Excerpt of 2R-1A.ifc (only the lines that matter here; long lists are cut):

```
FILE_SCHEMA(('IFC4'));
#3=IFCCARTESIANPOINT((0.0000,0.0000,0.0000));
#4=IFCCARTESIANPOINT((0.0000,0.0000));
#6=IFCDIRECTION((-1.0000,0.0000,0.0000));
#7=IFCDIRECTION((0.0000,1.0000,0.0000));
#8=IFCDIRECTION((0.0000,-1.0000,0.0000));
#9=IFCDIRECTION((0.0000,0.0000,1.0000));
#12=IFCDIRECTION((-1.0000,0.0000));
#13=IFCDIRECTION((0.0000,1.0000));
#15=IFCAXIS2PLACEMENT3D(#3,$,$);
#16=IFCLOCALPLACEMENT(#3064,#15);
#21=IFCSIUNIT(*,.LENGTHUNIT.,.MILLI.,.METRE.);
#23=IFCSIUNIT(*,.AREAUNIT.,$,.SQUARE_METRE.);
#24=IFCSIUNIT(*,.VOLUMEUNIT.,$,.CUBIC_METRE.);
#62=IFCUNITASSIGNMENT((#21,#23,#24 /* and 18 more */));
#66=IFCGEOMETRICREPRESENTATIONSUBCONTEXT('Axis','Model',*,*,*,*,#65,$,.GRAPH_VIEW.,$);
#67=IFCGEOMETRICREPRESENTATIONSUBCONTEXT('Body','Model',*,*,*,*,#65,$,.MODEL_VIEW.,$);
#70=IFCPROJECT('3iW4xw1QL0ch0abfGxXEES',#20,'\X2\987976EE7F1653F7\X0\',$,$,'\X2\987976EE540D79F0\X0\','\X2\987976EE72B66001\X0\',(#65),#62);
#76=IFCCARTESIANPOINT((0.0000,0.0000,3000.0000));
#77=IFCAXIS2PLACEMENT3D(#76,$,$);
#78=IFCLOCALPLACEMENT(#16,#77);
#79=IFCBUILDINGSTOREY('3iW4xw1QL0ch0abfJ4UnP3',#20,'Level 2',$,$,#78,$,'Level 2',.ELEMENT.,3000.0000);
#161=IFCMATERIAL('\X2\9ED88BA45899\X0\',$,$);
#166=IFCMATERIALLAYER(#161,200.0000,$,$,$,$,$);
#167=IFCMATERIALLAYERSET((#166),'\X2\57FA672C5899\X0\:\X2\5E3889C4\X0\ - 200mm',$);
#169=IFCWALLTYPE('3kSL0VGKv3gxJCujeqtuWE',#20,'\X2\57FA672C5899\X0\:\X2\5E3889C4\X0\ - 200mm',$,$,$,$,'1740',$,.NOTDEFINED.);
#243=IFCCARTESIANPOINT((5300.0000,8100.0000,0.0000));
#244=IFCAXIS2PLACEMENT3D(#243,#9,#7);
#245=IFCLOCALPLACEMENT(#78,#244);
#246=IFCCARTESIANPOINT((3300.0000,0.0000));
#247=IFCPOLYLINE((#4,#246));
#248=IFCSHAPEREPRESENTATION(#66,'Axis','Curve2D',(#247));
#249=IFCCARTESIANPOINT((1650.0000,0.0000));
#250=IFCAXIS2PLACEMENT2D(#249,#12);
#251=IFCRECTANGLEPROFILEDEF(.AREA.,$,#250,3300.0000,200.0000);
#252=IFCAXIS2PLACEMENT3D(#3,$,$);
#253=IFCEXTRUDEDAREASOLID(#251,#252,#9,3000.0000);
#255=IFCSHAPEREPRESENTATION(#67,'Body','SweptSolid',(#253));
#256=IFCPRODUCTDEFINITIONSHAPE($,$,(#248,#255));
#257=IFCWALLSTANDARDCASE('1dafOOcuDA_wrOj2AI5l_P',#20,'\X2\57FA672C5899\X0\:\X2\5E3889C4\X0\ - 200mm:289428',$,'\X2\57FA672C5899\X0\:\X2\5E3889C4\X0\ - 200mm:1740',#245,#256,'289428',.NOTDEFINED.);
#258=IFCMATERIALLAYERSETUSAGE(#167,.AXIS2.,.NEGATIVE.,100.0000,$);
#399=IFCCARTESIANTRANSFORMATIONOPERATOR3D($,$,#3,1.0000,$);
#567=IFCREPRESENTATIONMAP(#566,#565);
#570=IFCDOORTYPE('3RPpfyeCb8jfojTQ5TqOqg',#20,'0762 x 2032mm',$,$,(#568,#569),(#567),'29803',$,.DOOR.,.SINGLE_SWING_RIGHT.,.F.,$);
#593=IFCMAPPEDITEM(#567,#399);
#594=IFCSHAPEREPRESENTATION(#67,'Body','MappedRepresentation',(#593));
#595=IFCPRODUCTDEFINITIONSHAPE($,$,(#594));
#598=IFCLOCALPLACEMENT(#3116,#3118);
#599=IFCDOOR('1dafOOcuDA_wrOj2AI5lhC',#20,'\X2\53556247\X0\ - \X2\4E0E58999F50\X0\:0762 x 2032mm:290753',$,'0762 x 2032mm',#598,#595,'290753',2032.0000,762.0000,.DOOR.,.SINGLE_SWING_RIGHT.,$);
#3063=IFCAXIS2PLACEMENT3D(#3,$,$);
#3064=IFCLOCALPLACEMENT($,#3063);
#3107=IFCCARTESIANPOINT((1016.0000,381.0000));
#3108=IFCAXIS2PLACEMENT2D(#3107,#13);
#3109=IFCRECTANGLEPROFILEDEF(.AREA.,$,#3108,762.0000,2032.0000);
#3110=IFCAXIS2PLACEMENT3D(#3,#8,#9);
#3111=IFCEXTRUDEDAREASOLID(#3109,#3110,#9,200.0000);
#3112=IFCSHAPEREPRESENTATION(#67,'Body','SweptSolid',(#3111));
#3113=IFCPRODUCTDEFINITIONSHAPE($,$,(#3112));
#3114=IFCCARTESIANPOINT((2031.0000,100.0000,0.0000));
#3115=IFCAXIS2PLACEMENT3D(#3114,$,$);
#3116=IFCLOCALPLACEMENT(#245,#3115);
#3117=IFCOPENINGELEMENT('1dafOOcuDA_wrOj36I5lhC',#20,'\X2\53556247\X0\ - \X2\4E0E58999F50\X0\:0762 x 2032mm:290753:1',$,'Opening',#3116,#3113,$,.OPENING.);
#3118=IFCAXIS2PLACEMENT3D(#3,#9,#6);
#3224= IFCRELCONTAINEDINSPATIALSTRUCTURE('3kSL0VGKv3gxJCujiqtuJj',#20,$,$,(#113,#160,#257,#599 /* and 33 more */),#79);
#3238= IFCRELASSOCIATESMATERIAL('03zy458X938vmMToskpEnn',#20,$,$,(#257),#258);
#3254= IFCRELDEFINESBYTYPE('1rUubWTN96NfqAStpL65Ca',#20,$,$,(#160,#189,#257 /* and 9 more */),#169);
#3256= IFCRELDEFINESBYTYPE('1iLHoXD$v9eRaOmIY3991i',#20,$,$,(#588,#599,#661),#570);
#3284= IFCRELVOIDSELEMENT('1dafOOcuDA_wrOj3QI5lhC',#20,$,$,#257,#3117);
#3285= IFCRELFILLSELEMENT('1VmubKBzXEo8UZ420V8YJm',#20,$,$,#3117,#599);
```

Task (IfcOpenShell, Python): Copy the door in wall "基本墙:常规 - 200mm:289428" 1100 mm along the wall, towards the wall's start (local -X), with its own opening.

```python
import ifcopenshell
import ifcopenshell.api.feature
import ifcopenshell.api.geometry
import ifcopenshell.api.root
import ifcopenshell.geom
import ifcopenshell.util.element
import ifcopenshell.util.placement
import ifcopenshell.util.shape
import ifcopenshell.util.unit

model = ifcopenshell.open("2R-1A.ifc")
unit_scale = ifcopenshell.util.unit.calculate_unit_scale(model)
settings = ifcopenshell.geom.settings()


def volume(element):
    """Net volume in cubic metres, openings subtracted."""
    shape = ifcopenshell.geom.create_shape(settings, element)
    return ifcopenshell.util.shape.get_volume(shape.geometry)


def reuse_history(source, copy):
    """copy_class also copies each property set's owner history, people and application; keep the originals."""
    for rel in copy.IsDefinedBy:
        if rel.is_a("IfcRelDefinesByProperties") and (history := rel.RelatingPropertyDefinition.OwnerHistory):
            rel.RelatingPropertyDefinition.OwnerHistory = source.OwnerHistory
            ifcopenshell.util.element.remove_deep2(model, history)


door = model.by_id(599)
opening = door.FillsVoids[0].RelatingOpeningElement
wall = opening.VoidsElements[0].RelatingBuildingElement
before = volume(wall)
shift = ifcopenshell.util.placement.get_local_placement(wall.ObjectPlacement)[:3, 0] * -1.1 / unit_scale

# copy_class copies the void relationship, type, container and properties, but no geometry.
new_opening = ifcopenshell.api.root.copy_class(model, product=opening)
new_opening.Representation = ifcopenshell.util.element.copy_deep(
    model, opening.Representation, exclude=["IfcGeometricRepresentationContext", "IfcRepresentationMap"]
)
new_opening.Name = "单扇 - 与墙齐:0762 x 2032mm"
new_door = ifcopenshell.api.root.copy_class(model, product=door)
new_door.Representation = ifcopenshell.util.element.copy_deep(
    model, door.Representation, exclude=["IfcGeometricRepresentationContext", "IfcRepresentationMap"]
)
new_door.Name = "单扇 - 与墙齐:0762 x 2032mm"
new_door.Tag = None
reuse_history(door, new_door)
ifcopenshell.api.feature.add_filling(model, opening=new_opening, element=new_door)

for old, new in ((opening, new_opening), (door, new_door)):
    matrix = ifcopenshell.util.placement.get_local_placement(old.ObjectPlacement)
    matrix[:3, 3] += shift
    ifcopenshell.api.geometry.edit_object_placement(model, product=new, matrix=matrix, is_si=False)

after = volume(wall)

print(f"wall volume {before:.3f} -> {after:.3f} m3")

model.write("2R-1A_updated.ifc")
```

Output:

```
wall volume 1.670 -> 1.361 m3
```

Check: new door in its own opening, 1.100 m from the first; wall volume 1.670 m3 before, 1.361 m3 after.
